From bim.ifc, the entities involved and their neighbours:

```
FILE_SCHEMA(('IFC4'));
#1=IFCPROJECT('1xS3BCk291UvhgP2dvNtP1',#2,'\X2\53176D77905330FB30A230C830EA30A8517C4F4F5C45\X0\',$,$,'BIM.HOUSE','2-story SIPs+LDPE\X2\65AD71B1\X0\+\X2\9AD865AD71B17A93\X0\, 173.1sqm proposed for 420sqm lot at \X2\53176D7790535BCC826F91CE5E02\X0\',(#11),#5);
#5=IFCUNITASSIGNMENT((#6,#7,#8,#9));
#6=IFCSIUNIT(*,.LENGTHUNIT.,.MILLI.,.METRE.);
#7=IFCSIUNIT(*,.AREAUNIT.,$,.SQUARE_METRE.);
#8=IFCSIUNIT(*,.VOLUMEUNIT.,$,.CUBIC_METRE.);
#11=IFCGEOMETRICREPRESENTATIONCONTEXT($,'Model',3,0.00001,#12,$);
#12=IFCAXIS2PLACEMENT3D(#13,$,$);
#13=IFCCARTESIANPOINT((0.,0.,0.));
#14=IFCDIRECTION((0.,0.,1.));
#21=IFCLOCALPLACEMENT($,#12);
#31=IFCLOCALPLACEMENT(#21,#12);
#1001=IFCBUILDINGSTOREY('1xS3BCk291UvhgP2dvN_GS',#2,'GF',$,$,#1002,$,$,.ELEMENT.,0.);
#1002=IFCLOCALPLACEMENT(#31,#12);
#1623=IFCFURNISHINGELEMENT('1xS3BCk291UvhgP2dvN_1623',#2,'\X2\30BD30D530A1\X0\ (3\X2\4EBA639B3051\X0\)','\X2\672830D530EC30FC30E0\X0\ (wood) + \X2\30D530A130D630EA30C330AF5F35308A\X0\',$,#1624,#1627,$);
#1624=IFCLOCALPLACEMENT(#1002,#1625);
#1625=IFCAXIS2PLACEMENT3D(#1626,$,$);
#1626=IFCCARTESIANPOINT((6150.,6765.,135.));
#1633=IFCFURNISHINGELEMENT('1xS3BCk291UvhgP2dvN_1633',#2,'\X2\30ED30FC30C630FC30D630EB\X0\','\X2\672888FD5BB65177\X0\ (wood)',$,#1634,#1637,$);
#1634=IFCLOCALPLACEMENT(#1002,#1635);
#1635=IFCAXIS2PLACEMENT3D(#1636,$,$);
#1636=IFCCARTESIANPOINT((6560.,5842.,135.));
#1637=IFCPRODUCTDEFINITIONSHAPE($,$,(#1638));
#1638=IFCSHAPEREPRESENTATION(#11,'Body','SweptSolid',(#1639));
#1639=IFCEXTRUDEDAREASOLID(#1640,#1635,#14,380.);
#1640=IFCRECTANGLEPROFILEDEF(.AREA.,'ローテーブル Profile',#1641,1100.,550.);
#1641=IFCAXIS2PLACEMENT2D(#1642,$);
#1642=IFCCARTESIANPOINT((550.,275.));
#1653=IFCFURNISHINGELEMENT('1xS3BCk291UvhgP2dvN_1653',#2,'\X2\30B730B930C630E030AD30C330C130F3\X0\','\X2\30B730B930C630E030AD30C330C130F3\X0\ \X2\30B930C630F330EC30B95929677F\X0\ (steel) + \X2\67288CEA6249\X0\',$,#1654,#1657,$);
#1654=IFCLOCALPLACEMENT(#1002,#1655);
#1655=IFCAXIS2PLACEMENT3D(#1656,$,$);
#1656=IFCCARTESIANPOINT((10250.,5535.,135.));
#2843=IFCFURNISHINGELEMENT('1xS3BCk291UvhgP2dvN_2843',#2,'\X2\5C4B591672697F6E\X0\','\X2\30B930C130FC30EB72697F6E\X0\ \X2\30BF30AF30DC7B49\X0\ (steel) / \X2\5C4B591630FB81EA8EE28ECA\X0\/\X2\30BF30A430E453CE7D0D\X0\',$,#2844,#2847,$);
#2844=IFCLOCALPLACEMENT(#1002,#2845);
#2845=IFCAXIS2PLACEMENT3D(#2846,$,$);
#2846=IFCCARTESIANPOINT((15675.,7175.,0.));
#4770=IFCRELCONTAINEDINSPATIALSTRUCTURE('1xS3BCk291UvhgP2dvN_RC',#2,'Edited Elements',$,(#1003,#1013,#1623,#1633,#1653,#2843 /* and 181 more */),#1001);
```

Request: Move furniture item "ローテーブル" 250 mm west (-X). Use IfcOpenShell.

```python
import ifcopenshell
import ifcopenshell.api.geometry
import ifcopenshell.util.placement
import ifcopenshell.util.unit

model = ifcopenshell.open("bim.ifc")
unit_scale = ifcopenshell.util.unit.calculate_unit_scale(model)

item = model.by_guid("1xS3BCk291UvhgP2dvN_1633")
matrix = ifcopenshell.util.placement.get_local_placement(item.ObjectPlacement)
matrix[0, 3] -= 0.25 / unit_scale
ifcopenshell.api.geometry.edit_object_placement(model, product=item, matrix=matrix, is_si=False)

print(ifcopenshell.util.placement.get_local_placement(item.ObjectPlacement).round(3) + 0.0)

model.write("bim-out.ifc")
```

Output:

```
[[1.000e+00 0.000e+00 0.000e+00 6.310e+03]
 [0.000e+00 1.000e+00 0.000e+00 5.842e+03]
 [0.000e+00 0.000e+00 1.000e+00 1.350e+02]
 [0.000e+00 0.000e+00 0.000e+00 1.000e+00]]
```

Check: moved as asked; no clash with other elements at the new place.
